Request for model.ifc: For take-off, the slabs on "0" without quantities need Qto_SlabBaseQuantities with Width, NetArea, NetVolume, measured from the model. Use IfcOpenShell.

First a look at what the model holds.

```python
import ifcopenshell
import ifcopenshell.util.element
import ifcopenshell.util.unit

model = ifcopenshell.open("model.ifc")
print(model.schema)
for unit_type in ("LENGTHUNIT", "AREAUNIT", "VOLUMEUNIT"):
    print(unit_type, ifcopenshell.util.unit.calculate_unit_scale(model, unit_type))
storey = next(s for s in model.by_type("IfcBuildingStorey") if s.Name == "0")
slabs = [e for e in ifcopenshell.util.element.get_decomposition(storey) if e.is_a("IfcSlab")]
for e in sorted(slabs, key=lambda e: e.id()):
    print(e.id(), e.is_a(), e.Name, list(ifcopenshell.util.element.get_psets(e, qtos_only=True)), sep=" | ")
```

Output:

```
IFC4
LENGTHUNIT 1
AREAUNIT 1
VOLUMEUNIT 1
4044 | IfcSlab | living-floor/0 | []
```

```python
import ifcopenshell
import ifcopenshell.api.pset
import ifcopenshell.geom
import ifcopenshell.util.element
import ifcopenshell.util.shape
import ifcopenshell.util.unit

model = ifcopenshell.open("model.ifc")
unit_scale = ifcopenshell.util.unit.calculate_unit_scale(model)
area_scale = ifcopenshell.util.unit.calculate_unit_scale(model, "AREAUNIT")
volume_scale = ifcopenshell.util.unit.calculate_unit_scale(model, "VOLUMEUNIT")
settings = ifcopenshell.geom.settings()

storey = next(s for s in model.by_type("IfcBuildingStorey") if s.Name == "0")
slabs = [e for e in ifcopenshell.util.element.get_decomposition(storey) if e.is_a("IfcSlab")]

for e in sorted(slabs, key=lambda e: e.id()):
    if ifcopenshell.util.element.get_psets(e, qtos_only=True, should_inherit=False):
        continue
    # Geometry comes back in metres, in the element's own axes.
    shape = ifcopenshell.geom.create_shape(settings, e)
    values = {
        "Width": ifcopenshell.util.shape.get_z(shape.geometry) / unit_scale,
        "NetArea": ifcopenshell.util.shape.get_footprint_area(shape.geometry) / area_scale,
        "NetVolume": ifcopenshell.util.shape.get_volume(shape.geometry) / volume_scale,
    }
    qto = ifcopenshell.api.pset.add_qto(model, product=e, name="Qto_SlabBaseQuantities")
    ifcopenshell.api.pset.edit_qto(model, qto=qto, properties=values)
    print(e.id(), {k: round(v, 3) for k, v in values.items()})

model.write("model_updated.ifc")
```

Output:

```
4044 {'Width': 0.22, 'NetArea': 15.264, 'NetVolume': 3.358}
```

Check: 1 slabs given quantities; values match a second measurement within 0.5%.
